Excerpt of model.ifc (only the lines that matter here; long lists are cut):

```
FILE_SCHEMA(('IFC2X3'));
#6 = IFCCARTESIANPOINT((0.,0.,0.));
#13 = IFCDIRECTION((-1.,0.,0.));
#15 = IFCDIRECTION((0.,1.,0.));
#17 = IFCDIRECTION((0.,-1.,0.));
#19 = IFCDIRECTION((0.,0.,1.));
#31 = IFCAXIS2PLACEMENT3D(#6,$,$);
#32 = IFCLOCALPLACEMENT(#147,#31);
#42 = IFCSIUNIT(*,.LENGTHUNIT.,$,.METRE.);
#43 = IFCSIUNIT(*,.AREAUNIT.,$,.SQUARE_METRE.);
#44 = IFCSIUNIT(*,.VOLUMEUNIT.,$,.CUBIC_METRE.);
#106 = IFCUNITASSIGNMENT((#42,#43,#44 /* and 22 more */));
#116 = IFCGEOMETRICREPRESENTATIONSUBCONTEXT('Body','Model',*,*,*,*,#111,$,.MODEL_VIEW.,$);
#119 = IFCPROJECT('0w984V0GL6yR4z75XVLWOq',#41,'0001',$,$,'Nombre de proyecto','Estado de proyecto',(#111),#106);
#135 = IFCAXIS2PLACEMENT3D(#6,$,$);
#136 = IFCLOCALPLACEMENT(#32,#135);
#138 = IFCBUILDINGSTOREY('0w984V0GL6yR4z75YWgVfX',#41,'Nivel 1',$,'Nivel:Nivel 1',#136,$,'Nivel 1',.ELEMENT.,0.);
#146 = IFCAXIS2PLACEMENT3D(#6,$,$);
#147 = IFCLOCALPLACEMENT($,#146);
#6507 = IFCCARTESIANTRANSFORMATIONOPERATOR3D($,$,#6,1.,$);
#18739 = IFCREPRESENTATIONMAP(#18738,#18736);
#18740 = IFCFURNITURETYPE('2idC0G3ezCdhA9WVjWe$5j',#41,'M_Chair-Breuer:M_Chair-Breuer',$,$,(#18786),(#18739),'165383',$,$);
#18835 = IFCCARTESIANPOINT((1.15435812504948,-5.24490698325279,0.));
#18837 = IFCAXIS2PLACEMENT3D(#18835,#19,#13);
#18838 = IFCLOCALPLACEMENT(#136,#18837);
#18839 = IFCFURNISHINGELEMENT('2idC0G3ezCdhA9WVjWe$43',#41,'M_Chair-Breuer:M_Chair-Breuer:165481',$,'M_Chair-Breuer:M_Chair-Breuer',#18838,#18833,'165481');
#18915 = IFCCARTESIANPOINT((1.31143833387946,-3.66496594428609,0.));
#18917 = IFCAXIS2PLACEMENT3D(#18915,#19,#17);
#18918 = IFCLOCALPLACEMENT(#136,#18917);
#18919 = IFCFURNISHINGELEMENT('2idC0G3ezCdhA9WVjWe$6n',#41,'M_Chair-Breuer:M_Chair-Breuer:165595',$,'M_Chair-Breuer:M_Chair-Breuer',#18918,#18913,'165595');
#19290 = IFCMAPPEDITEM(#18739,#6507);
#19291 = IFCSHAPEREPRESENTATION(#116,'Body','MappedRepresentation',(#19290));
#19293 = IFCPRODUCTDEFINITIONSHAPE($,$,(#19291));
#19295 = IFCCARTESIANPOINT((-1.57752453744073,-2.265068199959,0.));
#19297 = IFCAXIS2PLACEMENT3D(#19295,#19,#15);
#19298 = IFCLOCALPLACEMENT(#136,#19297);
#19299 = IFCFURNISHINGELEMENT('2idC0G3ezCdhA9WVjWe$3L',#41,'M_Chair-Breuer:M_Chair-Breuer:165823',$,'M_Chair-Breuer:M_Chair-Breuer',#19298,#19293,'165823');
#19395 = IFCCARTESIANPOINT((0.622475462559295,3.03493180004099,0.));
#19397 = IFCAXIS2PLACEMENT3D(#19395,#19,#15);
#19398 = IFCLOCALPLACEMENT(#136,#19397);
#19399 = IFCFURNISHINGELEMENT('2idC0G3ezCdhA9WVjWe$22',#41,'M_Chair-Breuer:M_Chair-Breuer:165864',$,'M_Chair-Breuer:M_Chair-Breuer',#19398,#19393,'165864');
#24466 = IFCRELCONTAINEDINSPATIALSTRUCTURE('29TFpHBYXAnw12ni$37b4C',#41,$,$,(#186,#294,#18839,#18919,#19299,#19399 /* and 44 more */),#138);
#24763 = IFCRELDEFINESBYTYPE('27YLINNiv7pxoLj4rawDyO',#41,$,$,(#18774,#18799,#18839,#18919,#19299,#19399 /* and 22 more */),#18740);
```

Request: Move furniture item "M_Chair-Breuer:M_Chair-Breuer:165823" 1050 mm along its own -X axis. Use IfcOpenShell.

```python
import ifcopenshell
import ifcopenshell.api.geometry
import ifcopenshell.util.placement
import ifcopenshell.util.unit

model = ifcopenshell.open("model.ifc")
unit_scale = ifcopenshell.util.unit.calculate_unit_scale(model)

item = model.by_guid("2idC0G3ezCdhA9WVjWe$3L")
matrix = ifcopenshell.util.placement.get_local_placement(item.ObjectPlacement)
matrix[:3, 3] -= matrix[:3, 0] * 1.05 / unit_scale
ifcopenshell.api.geometry.edit_object_placement(model, product=item, matrix=matrix, is_si=False)

print(ifcopenshell.util.placement.get_local_placement(item.ObjectPlacement).round(3) + 0.0)

model.write("model_edited.ifc")
```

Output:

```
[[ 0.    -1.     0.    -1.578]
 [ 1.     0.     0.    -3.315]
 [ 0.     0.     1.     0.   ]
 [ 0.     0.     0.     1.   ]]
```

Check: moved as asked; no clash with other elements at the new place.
